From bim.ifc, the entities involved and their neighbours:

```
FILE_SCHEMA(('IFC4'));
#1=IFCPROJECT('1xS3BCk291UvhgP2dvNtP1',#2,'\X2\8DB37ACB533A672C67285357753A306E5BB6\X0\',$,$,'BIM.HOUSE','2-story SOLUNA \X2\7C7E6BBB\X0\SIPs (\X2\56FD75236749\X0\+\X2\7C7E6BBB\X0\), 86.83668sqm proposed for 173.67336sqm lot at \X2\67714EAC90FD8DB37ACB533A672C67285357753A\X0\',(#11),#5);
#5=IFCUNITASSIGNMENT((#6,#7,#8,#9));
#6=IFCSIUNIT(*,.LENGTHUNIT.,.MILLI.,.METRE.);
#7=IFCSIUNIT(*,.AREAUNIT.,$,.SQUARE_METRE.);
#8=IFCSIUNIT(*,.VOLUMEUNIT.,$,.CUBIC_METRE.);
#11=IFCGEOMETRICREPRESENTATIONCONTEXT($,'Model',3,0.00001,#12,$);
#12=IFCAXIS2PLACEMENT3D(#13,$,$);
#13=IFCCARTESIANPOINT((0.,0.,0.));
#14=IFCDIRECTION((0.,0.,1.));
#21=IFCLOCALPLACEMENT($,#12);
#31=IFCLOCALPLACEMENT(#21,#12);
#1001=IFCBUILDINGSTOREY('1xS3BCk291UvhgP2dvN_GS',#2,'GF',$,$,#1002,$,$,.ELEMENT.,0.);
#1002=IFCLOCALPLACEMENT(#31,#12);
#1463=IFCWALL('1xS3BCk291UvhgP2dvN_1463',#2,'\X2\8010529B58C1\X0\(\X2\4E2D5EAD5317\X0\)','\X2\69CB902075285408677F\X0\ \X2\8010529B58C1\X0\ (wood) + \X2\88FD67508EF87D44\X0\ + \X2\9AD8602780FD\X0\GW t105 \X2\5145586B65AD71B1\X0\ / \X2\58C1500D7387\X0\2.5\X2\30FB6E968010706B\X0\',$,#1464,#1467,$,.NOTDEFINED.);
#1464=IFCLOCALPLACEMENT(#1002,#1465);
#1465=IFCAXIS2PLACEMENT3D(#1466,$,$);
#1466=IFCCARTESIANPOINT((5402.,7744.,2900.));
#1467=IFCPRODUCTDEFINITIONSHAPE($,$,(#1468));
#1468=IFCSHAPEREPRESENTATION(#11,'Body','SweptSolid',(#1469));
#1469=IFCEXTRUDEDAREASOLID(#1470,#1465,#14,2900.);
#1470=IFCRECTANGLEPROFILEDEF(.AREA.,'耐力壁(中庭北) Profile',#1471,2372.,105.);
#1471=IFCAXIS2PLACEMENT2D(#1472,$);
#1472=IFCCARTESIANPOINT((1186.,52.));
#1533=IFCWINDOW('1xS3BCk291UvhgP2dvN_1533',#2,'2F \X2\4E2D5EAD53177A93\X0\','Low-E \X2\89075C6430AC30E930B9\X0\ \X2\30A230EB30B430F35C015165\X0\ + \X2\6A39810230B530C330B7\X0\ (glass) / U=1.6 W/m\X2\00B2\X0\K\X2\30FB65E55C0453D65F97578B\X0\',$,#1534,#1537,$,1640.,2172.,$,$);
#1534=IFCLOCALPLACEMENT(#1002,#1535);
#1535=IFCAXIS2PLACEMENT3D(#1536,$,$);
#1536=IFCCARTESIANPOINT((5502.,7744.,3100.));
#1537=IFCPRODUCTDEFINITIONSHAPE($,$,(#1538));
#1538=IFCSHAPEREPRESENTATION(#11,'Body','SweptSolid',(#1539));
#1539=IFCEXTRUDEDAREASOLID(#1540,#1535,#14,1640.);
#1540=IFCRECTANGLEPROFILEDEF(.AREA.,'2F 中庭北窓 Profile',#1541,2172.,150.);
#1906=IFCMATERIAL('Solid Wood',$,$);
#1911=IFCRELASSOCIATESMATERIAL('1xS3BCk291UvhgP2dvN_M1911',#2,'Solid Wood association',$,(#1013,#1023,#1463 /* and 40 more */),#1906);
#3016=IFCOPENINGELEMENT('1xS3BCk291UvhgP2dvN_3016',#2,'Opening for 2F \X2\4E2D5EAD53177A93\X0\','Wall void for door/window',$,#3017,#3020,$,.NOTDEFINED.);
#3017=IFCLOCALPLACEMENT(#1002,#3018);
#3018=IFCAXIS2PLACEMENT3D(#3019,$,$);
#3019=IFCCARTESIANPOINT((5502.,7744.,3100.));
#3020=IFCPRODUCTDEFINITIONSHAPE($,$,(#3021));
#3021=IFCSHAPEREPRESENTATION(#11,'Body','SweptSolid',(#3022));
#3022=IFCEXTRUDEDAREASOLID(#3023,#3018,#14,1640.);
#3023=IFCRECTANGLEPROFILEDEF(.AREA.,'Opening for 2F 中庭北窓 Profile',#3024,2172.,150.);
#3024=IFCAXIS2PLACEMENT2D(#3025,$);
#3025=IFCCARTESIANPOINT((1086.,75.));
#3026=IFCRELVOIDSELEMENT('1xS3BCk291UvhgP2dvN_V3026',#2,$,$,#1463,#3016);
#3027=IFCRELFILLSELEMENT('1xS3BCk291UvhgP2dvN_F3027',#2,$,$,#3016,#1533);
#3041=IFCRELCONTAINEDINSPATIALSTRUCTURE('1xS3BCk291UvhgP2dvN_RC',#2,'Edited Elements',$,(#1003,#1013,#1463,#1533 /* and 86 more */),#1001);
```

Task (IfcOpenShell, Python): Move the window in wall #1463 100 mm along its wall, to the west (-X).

```python
import ifcopenshell
import ifcopenshell.api.geometry
import ifcopenshell.util.placement
import ifcopenshell.util.unit

model = ifcopenshell.open("bim.ifc")
unit_scale = ifcopenshell.util.unit.calculate_unit_scale(model)

window = model.by_guid("1xS3BCk291UvhgP2dvN_1533")
opening = window.FillsVoids[0].RelatingOpeningElement
wall = opening.VoidsElements[0].RelatingBuildingElement

wall_matrix = ifcopenshell.util.placement.get_local_placement(wall.ObjectPlacement)
shift = wall_matrix[:3, 0] * -0.1 / unit_scale
before = ifcopenshell.util.placement.get_local_placement(window.ObjectPlacement)[:3, 3].copy()

# The window is not placed relative to its opening, so move both.
for product in (opening, window):
    matrix = ifcopenshell.util.placement.get_local_placement(product.ObjectPlacement)
    matrix[:3, 3] += shift
    ifcopenshell.api.geometry.edit_object_placement(model, product=product, matrix=matrix, is_si=False)

after = ifcopenshell.util.placement.get_local_placement(window.ObjectPlacement)[:3, 3]
print("window moved by", (after - before).round(3) + 0.0)

model.write("bim_updated.ifc")
```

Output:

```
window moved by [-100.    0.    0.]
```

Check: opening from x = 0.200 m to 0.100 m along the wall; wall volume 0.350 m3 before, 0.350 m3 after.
